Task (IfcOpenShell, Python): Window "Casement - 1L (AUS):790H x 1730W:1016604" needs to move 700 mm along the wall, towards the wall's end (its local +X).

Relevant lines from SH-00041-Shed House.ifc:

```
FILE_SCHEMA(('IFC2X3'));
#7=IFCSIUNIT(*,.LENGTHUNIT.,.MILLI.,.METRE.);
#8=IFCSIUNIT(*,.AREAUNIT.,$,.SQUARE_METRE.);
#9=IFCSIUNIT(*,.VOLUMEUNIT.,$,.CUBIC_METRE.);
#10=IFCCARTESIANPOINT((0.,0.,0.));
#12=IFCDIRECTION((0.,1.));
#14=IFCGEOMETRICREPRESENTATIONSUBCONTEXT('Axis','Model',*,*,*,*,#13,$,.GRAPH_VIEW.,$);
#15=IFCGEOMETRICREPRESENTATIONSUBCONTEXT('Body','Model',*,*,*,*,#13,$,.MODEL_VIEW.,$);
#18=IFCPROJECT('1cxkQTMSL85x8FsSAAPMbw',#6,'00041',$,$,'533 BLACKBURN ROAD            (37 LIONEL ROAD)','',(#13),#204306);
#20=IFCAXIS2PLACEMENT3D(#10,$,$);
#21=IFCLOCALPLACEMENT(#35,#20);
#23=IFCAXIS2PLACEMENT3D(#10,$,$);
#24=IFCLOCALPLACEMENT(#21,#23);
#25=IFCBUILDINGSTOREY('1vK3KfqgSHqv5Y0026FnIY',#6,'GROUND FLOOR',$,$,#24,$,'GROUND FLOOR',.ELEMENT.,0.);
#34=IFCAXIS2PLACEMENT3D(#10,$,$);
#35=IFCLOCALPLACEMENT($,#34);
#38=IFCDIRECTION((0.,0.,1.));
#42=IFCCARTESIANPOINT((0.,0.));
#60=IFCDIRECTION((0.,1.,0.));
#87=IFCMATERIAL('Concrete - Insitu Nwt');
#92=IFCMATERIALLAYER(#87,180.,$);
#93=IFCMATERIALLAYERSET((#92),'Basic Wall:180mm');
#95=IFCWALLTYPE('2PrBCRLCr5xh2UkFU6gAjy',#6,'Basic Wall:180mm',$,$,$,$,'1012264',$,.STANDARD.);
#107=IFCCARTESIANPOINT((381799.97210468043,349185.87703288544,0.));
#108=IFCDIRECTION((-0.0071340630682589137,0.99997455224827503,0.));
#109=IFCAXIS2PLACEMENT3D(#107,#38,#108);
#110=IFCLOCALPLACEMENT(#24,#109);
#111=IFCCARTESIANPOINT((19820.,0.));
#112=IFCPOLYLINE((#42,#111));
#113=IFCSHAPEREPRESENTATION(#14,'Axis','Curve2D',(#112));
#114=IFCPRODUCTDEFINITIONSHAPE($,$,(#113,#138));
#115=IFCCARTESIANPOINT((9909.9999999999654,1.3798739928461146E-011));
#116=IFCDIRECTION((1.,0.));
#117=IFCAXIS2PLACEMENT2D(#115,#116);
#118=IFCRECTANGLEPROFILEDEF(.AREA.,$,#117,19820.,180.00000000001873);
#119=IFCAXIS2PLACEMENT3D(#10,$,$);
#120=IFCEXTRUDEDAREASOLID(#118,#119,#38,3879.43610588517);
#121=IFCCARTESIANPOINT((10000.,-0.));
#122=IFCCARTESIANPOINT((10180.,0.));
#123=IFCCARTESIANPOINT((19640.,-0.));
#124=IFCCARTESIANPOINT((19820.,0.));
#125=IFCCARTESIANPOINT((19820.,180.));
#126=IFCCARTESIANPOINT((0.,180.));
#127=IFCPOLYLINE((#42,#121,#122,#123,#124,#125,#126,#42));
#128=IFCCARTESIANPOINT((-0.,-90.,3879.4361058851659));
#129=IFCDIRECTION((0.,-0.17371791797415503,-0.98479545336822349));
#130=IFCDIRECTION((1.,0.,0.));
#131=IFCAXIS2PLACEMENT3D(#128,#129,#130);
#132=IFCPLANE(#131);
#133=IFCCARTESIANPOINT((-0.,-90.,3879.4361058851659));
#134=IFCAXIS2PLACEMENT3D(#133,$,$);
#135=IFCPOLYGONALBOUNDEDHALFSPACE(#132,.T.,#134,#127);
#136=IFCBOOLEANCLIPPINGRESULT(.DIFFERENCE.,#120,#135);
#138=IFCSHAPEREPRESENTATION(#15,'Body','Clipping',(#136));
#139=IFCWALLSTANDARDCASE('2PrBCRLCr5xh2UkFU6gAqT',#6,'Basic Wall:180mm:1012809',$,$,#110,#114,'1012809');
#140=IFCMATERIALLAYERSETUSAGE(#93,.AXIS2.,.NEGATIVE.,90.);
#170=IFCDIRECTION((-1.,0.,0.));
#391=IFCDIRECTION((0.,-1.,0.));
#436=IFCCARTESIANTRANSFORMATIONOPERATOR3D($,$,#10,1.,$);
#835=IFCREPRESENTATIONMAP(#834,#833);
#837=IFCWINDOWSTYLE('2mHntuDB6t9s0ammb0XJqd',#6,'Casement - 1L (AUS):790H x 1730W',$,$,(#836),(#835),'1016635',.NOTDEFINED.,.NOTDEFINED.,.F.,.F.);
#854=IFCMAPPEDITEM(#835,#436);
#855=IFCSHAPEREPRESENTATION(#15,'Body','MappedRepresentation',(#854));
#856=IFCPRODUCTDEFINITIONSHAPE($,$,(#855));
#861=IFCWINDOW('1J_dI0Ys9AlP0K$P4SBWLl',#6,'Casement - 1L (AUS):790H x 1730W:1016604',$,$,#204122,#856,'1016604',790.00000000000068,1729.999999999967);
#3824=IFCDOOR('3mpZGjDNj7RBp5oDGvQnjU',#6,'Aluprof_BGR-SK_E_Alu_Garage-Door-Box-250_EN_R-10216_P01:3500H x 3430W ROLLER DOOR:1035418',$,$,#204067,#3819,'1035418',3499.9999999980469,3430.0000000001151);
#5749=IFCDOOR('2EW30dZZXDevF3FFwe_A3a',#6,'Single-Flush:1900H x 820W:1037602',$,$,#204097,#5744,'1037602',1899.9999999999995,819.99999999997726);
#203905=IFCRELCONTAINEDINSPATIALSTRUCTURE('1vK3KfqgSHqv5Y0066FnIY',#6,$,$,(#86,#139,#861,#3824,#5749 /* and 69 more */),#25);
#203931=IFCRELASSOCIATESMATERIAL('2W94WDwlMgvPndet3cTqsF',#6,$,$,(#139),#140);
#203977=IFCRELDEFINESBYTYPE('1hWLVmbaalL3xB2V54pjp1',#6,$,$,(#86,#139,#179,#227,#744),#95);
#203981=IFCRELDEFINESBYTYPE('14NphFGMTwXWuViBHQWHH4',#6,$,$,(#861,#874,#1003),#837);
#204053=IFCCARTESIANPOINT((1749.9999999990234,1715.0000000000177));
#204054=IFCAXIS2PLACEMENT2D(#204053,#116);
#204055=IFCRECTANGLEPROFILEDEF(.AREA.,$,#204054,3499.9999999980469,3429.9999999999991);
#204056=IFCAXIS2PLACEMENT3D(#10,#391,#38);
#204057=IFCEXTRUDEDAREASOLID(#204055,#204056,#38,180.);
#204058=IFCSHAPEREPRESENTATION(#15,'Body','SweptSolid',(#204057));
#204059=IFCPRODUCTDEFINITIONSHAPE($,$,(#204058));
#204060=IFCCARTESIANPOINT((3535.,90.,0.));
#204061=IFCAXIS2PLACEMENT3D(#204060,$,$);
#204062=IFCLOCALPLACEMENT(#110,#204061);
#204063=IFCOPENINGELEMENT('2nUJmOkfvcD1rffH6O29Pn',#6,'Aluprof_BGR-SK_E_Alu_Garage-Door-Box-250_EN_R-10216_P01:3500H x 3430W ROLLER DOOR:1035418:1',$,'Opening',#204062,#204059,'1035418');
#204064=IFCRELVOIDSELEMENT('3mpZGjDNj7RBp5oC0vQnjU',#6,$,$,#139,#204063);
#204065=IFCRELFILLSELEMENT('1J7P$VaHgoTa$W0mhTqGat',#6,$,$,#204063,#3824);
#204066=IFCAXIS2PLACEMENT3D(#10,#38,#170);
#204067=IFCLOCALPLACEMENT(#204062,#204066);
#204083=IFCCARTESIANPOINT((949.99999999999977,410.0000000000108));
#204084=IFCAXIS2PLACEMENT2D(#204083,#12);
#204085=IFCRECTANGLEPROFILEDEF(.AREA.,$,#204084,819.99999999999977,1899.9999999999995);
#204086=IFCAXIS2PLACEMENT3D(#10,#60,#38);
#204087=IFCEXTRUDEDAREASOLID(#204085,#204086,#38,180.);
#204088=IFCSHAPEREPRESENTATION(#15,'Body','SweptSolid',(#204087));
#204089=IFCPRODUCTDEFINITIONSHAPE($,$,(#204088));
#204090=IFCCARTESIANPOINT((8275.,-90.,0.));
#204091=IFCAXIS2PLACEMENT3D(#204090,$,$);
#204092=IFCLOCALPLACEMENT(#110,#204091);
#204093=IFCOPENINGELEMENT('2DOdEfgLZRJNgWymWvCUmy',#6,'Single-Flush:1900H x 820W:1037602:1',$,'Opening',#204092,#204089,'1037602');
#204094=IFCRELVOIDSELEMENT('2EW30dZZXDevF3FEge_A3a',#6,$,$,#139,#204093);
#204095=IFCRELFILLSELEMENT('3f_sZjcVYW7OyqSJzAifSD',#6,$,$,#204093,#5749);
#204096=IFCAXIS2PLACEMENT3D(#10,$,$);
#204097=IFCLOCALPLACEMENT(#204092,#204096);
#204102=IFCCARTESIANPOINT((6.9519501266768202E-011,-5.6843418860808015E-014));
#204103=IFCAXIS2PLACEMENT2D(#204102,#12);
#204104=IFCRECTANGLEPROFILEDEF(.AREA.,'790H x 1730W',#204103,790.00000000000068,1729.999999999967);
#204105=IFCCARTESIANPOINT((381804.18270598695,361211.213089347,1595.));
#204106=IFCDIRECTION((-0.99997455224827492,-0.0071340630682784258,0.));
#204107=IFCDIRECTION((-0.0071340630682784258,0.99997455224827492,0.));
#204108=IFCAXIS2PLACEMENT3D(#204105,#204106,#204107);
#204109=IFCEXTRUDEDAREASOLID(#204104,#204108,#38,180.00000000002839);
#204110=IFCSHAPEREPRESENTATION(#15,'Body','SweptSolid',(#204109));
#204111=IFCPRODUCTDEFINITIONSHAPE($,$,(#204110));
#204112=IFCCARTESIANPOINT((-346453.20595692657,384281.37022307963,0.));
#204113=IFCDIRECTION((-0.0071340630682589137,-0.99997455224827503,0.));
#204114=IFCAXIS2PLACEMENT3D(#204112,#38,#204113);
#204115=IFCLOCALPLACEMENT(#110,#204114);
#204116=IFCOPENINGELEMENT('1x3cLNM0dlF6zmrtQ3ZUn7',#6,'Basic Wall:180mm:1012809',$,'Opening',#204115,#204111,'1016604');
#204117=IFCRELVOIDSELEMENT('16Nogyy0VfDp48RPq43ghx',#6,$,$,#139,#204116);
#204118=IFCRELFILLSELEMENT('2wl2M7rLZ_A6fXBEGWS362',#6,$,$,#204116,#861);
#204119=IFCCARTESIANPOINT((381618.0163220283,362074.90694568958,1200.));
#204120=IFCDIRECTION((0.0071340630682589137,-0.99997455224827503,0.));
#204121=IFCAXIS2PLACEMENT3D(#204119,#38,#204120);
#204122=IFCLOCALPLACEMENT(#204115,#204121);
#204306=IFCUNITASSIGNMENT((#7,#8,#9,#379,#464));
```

```python
import ifcopenshell
import ifcopenshell.api.geometry
import ifcopenshell.util.placement

model = ifcopenshell.open("SH-00041-Shed House.ifc")

window = model.by_guid("1J_dI0Ys9AlP0K$P4SBWLl")
opening = window.FillsVoids[0].RelatingOpeningElement
wall = opening.VoidsElements[0].RelatingBuildingElement

wall_matrix = ifcopenshell.util.placement.get_local_placement(wall.ObjectPlacement)
shift = wall_matrix[:3, 0] * 700.0
before = ifcopenshell.util.placement.get_local_placement(window.ObjectPlacement)[:3, 3].copy()

# The window is placed relative to its opening, so it follows when the opening moves.
matrix = ifcopenshell.util.placement.get_local_placement(opening.ObjectPlacement)
matrix[:3, 3] += shift
ifcopenshell.api.geometry.edit_object_placement(
    model, product=opening, matrix=matrix, is_si=False, should_transform_children=True
)

after = ifcopenshell.util.placement.get_local_placement(window.ObjectPlacement)[:3, 3]
print("window moved by", (after - before).round(3) + 0.0)

model.write("SH-00041-Shed House_v2.ifc")
```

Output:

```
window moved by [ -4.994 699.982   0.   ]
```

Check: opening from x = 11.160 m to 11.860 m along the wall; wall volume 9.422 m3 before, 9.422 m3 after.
